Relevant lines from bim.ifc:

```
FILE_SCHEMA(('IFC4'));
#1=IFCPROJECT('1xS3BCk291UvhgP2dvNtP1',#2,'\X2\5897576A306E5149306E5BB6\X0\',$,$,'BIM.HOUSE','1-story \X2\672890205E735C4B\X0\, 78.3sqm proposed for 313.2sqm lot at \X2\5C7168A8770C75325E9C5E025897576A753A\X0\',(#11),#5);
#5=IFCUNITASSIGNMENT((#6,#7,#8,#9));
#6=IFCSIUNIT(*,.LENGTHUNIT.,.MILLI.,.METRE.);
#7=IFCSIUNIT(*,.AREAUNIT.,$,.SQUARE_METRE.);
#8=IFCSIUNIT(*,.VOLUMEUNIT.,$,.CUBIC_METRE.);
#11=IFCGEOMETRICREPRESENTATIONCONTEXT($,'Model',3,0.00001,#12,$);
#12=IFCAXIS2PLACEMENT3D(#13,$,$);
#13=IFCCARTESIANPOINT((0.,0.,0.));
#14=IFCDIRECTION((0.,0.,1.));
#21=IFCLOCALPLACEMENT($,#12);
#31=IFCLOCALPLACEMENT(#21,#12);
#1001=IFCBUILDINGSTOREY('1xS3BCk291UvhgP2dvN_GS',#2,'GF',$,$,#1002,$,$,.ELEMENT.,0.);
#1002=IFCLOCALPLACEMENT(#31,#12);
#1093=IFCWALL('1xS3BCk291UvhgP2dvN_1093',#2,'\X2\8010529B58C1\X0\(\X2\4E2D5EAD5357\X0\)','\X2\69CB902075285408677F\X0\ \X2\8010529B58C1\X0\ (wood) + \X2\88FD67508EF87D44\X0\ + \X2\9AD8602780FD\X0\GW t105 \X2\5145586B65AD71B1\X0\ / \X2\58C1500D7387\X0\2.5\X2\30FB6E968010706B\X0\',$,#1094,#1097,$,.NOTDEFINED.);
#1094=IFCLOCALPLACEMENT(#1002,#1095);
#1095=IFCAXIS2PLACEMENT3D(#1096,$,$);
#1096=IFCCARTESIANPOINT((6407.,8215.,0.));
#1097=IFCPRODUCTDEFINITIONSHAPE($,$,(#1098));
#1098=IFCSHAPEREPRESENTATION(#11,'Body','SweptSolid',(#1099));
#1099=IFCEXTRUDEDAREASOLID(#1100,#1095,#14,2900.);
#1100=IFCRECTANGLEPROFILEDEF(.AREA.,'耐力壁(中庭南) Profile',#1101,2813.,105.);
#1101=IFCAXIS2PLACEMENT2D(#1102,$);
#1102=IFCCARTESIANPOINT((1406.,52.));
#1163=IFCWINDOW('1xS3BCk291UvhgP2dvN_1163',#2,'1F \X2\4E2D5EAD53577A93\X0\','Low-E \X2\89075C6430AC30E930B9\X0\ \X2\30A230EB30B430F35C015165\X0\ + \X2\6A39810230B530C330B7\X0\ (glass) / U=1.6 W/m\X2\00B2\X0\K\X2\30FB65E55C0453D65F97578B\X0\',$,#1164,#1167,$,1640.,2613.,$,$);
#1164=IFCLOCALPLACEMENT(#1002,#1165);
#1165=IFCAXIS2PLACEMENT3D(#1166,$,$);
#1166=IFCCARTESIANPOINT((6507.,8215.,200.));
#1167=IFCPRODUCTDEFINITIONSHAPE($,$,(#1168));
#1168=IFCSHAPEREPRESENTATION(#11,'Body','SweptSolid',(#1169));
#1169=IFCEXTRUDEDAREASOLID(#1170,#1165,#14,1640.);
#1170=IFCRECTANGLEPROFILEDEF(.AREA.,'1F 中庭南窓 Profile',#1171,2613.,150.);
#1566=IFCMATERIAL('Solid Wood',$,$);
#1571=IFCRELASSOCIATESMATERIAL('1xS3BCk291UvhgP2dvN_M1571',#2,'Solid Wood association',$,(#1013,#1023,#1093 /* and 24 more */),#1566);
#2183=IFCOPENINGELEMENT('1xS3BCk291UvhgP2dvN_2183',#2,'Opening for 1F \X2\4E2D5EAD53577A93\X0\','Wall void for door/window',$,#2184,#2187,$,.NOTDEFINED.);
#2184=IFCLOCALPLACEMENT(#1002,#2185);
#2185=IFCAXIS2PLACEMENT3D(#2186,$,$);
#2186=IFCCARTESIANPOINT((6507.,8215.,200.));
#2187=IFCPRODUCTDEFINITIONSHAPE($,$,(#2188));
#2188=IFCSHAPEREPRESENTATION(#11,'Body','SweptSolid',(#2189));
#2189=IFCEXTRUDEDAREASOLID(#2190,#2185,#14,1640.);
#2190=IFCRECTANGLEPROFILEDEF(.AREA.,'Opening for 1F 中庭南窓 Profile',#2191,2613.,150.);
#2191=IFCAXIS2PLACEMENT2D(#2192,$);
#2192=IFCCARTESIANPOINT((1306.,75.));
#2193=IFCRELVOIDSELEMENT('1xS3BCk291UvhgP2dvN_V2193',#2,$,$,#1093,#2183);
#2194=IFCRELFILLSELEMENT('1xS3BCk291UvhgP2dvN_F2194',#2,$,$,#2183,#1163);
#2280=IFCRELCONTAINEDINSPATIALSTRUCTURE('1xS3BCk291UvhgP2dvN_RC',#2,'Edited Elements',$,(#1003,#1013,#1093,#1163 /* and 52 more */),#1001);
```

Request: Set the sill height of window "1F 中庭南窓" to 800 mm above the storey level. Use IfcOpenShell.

```python
import numpy as np
import ifcopenshell
import ifcopenshell.api.geometry
import ifcopenshell.geom
import ifcopenshell.util.element
import ifcopenshell.util.placement
import ifcopenshell.util.shape
import ifcopenshell.util.unit

model = ifcopenshell.open("bim.ifc")
unit_scale = ifcopenshell.util.unit.calculate_unit_scale(model)

window = model.by_guid("1xS3BCk291UvhgP2dvN_1163")
opening = window.FillsVoids[0].RelatingOpeningElement
storey = ifcopenshell.util.element.get_container(window, ifc_class="IfcBuildingStorey")
level = ifcopenshell.util.placement.get_local_placement(storey.ObjectPlacement)[2, 3]

# The opening's origin need not be at the sill, so measure its lowest point.
shape = ifcopenshell.geom.create_shape(ifcopenshell.geom.settings(), opening)
bottom = ifcopenshell.util.shape.get_shape_bottom_elevation(shape, shape.geometry) / unit_scale
dz = level + 0.8 / unit_scale - bottom

shift = np.array([0.0, 0.0, dz])
# The window is not placed relative to its opening, so move both.
for product in (opening, window):
    matrix = ifcopenshell.util.placement.get_local_placement(product.ObjectPlacement)
    matrix[:3, 3] += shift
    ifcopenshell.api.geometry.edit_object_placement(model, product=product, matrix=matrix, is_si=False)

print(f"moved by {dz * unit_scale:+.3f} m")

model.write("bim-out.ifc")
```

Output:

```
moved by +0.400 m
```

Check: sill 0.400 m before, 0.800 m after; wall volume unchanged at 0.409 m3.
